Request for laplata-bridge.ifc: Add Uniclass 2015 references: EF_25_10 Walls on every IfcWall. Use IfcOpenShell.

First a look at what the model holds.

```python
import ifcopenshell

model = ifcopenshell.open("laplata-bridge.ifc")
print(model.schema)
print("classifications:", [c.Name for c in model.by_type("IfcClassification")])
for ifc_class in ("IfcDoor", "IfcRoof", "IfcStair", "IfcWall", "IfcWindow"):
    print(ifc_class, len(model.by_type(ifc_class)))
```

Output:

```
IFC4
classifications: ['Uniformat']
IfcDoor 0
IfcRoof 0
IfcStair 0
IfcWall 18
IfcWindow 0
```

```python
import ifcopenshell
import ifcopenshell.api.classification

model = ifcopenshell.open("laplata-bridge.ifc")

system = ifcopenshell.api.classification.add_classification(model, classification="Uniclass 2015")

codes = {
    "IfcWall": ("EF_25_10", "Walls"),
}
for ifc_class, (code, name) in codes.items():
    products = model.by_type(ifc_class)
    ifcopenshell.api.classification.add_reference(
        model, products=products, classification=system, identification=code, name=name
    )
    print(code, len(products))

model.write("laplata-bridge-out.ifc")
```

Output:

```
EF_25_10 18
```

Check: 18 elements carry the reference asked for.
